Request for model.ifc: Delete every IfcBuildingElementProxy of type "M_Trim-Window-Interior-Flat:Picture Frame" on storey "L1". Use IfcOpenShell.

First a look at what the model holds.

```python
import ifcopenshell
import ifcopenshell.util.element

model = ifcopenshell.open("model.ifc")
print(model.schema)
storey = next(s for s in model.by_type("IfcBuildingStorey") if s.Name == "L1")
proxies = [e for e in ifcopenshell.util.element.get_decomposition(storey) if e.is_a("IfcBuildingElementProxy")]
seen = {}
for e in proxies:
    element_type = ifcopenshell.util.element.get_type(e)
    name = element_type.Name if element_type not in (None, e) else None
    seen[name] = seen.get(name, 0) + 1
for name, count in sorted(seen.items(), key=str):
    print(count, "x", name)
```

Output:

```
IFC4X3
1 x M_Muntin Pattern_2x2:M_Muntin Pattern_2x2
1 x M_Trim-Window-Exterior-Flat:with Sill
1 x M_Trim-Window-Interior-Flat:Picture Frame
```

```python
import ifcopenshell
import ifcopenshell.api.root
import ifcopenshell.util.element

model = ifcopenshell.open("model.ifc")

storey = next(s for s in model.by_type("IfcBuildingStorey") if s.Name == "L1")
proxies = [e for e in ifcopenshell.util.element.get_decomposition(storey) if e.is_a("IfcBuildingElementProxy")]
targets = [e for e in proxies if (t := ifcopenshell.util.element.get_type(e)) not in (None, e) and t.Name == "M_Trim-Window-Interior-Flat:Picture Frame"]

for e in targets:
    ifcopenshell.api.root.remove_product(model, product=e)
print(len(targets), "removed")

model.write("model_v2.ifc")
```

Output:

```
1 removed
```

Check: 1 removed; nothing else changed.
